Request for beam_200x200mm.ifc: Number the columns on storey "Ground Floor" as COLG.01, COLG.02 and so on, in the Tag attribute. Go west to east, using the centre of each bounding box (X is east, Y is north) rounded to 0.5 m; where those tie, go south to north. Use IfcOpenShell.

First a look at what the model holds.

```python
import ifcopenshell
import ifcopenshell.util.element
import ifcopenshell.util.placement

model = ifcopenshell.open("beam_200x200mm.ifc")
print(model.schema)
storey = next(s for s in model.by_type("IfcBuildingStorey") if s.Name == "Ground Floor")
columns = [e for e in ifcopenshell.util.element.get_decomposition(storey) if e.is_a("IfcColumn")]
for e in sorted(columns, key=lambda e: e.id()):
    origin = ifcopenshell.util.placement.get_local_placement(e.ObjectPlacement)[:3, 3]
    print(e.id(), e.Tag, e.Name, origin.round(2) + 0.0, sep=" | ")
```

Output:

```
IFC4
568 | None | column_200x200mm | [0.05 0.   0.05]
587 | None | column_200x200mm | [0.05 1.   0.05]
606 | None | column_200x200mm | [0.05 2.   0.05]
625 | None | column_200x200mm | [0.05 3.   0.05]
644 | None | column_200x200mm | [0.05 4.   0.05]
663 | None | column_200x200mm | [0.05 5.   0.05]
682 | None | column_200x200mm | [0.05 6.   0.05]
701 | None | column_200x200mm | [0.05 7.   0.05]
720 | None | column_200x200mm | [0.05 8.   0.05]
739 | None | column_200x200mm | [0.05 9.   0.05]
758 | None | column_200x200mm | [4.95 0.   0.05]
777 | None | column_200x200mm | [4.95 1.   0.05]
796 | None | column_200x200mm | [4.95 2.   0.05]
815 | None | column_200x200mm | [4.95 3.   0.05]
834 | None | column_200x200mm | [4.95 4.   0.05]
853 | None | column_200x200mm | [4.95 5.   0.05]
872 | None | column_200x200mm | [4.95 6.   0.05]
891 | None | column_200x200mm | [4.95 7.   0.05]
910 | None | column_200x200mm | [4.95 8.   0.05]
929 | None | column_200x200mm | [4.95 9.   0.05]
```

```python
import ifcopenshell
import ifcopenshell.geom
import ifcopenshell.util.element
import ifcopenshell.util.shape

model = ifcopenshell.open("beam_200x200mm.ifc")
settings = ifcopenshell.geom.settings()
settings.set("use-world-coords", True)


def centre(element):
    shape = ifcopenshell.geom.create_shape(settings, element)
    return ifcopenshell.util.shape.get_bbox_centroid(shape.geometry)


storey = next(s for s in model.by_type("IfcBuildingStorey") if s.Name == "Ground Floor")
columns = [e for e in ifcopenshell.util.element.get_decomposition(storey) if e.is_a("IfcColumn")]

# Insertion points can sit at a corner or the storey origin, so sort by the geometry (in metres).
centres = {e: centre(e) for e in columns}
columns.sort(key=lambda e: (round(centres[e][0] / 0.5), centres[e][1]))

for i, e in enumerate(columns, start=1):
    number = f"COLG.{i:02d}"
    e.Tag = number
    print(e.id(), number)

model.write("beam_200x200mm_v2.ifc")
```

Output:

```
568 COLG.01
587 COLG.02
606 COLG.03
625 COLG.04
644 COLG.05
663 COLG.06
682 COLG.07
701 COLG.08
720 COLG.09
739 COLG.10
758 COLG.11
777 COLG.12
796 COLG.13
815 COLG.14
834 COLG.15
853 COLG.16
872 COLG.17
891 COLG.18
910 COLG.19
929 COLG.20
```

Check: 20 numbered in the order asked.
